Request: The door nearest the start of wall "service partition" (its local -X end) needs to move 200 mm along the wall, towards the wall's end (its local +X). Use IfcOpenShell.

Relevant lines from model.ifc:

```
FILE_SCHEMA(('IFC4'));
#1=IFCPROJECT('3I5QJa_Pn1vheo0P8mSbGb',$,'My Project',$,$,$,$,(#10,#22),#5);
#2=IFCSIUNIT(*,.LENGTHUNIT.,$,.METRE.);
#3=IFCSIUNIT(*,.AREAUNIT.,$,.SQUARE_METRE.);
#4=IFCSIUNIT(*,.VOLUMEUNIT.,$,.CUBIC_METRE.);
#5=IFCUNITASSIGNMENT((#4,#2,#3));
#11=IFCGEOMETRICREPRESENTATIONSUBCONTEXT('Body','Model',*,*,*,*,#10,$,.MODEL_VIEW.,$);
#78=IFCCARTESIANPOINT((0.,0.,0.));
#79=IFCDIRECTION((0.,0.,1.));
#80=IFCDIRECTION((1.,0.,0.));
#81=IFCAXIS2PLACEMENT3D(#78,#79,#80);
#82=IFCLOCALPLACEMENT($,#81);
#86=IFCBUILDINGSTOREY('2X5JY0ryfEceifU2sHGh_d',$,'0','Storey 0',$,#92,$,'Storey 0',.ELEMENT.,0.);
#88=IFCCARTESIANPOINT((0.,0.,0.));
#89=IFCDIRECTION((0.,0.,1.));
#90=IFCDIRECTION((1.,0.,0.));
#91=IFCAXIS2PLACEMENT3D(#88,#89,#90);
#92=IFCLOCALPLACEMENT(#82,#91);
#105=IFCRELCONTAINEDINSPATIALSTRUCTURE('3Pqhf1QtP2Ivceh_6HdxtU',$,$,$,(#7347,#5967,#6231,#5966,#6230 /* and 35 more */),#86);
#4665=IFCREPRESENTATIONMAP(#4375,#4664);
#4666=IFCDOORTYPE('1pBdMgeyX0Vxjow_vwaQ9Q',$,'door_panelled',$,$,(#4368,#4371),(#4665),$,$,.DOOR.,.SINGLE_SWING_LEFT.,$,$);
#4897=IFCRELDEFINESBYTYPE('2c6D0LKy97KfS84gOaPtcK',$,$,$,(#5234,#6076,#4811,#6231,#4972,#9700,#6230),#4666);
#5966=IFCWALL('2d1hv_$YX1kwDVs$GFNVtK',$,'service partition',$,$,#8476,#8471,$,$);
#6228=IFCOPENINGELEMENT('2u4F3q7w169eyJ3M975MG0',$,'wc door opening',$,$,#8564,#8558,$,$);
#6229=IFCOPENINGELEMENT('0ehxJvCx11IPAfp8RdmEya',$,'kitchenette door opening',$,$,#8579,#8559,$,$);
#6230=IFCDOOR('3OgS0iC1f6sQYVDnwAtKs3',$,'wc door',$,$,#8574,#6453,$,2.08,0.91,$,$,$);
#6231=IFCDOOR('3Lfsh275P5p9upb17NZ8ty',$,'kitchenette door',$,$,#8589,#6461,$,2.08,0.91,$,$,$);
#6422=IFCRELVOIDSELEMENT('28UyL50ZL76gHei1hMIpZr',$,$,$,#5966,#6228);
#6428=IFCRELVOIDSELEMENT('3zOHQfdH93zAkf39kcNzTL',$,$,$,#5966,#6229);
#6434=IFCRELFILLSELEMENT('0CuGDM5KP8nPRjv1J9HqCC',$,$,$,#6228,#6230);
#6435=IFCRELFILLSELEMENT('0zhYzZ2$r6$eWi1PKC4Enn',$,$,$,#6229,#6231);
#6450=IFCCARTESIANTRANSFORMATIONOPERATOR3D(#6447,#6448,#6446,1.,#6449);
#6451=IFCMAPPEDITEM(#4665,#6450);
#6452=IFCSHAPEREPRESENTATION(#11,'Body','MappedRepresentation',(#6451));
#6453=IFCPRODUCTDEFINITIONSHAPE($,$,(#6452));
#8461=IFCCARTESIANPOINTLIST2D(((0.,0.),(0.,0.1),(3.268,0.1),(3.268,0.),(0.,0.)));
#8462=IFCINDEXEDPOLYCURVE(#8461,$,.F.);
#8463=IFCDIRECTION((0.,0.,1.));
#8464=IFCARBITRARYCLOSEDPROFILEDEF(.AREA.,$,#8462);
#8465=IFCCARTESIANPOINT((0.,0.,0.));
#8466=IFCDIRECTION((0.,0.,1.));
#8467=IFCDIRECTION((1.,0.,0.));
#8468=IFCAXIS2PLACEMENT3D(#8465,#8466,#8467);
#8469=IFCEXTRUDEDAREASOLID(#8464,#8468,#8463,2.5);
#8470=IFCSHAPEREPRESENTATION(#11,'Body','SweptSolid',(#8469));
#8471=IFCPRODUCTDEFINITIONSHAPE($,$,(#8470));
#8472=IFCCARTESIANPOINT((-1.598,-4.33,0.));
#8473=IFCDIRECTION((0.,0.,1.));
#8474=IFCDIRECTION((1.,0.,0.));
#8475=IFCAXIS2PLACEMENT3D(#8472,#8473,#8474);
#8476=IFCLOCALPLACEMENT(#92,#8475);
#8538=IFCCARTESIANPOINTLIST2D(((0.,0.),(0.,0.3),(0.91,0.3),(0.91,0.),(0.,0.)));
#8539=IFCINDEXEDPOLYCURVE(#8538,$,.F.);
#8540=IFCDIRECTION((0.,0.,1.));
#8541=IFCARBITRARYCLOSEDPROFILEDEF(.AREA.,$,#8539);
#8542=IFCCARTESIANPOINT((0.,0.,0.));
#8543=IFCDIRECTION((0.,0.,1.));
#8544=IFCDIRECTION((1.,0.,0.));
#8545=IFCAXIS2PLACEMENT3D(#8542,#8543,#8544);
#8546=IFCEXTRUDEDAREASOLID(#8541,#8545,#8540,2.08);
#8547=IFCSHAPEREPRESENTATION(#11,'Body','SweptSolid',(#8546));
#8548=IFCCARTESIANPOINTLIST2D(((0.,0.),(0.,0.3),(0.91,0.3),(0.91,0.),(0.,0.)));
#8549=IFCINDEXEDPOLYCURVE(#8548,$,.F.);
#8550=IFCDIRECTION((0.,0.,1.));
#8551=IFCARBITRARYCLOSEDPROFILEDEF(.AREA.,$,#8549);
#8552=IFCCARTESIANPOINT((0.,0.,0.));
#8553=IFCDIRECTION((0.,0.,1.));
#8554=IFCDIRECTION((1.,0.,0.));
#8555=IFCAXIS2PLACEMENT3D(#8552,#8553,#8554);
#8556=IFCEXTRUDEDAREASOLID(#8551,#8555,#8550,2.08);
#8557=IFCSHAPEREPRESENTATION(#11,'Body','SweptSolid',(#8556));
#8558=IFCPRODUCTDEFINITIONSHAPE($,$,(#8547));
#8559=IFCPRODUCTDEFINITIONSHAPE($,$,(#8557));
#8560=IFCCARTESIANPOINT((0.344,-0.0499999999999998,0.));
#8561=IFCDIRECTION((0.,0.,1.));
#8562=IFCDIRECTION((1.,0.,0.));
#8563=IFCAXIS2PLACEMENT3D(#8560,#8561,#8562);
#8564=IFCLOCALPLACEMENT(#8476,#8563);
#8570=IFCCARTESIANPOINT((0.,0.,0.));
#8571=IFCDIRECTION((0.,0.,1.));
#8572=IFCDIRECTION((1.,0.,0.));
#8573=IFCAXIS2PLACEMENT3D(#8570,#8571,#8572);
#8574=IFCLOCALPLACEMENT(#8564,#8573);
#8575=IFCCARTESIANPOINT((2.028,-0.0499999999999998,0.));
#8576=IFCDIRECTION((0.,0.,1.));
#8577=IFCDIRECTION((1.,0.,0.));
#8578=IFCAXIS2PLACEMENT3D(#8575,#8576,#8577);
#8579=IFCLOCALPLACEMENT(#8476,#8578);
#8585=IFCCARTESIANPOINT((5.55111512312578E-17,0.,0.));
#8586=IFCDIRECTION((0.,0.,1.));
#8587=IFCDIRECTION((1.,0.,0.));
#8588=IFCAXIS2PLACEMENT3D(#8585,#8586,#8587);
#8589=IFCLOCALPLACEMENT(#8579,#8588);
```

```python
import ifcopenshell
import ifcopenshell.api.geometry
import ifcopenshell.util.placement
import ifcopenshell.util.unit

model = ifcopenshell.open("model.ifc")
unit_scale = ifcopenshell.util.unit.calculate_unit_scale(model)

door = model.by_guid("3OgS0iC1f6sQYVDnwAtKs3")
opening = door.FillsVoids[0].RelatingOpeningElement
wall = opening.VoidsElements[0].RelatingBuildingElement

wall_matrix = ifcopenshell.util.placement.get_local_placement(wall.ObjectPlacement)
shift = wall_matrix[:3, 0] * 0.2 / unit_scale
before = ifcopenshell.util.placement.get_local_placement(door.ObjectPlacement)[:3, 3].copy()

# The door is placed relative to its opening, so it follows when the opening moves.
matrix = ifcopenshell.util.placement.get_local_placement(opening.ObjectPlacement)
matrix[:3, 3] += shift
ifcopenshell.api.geometry.edit_object_placement(
    model, product=opening, matrix=matrix, is_si=False, should_transform_children=True
)

after = ifcopenshell.util.placement.get_local_placement(door.ObjectPlacement)[:3, 3]
print("door moved by", (after - before).round(3) + 0.0)

model.write("model_edited.ifc")
```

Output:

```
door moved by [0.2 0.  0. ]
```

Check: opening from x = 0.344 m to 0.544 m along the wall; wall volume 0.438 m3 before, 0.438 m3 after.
